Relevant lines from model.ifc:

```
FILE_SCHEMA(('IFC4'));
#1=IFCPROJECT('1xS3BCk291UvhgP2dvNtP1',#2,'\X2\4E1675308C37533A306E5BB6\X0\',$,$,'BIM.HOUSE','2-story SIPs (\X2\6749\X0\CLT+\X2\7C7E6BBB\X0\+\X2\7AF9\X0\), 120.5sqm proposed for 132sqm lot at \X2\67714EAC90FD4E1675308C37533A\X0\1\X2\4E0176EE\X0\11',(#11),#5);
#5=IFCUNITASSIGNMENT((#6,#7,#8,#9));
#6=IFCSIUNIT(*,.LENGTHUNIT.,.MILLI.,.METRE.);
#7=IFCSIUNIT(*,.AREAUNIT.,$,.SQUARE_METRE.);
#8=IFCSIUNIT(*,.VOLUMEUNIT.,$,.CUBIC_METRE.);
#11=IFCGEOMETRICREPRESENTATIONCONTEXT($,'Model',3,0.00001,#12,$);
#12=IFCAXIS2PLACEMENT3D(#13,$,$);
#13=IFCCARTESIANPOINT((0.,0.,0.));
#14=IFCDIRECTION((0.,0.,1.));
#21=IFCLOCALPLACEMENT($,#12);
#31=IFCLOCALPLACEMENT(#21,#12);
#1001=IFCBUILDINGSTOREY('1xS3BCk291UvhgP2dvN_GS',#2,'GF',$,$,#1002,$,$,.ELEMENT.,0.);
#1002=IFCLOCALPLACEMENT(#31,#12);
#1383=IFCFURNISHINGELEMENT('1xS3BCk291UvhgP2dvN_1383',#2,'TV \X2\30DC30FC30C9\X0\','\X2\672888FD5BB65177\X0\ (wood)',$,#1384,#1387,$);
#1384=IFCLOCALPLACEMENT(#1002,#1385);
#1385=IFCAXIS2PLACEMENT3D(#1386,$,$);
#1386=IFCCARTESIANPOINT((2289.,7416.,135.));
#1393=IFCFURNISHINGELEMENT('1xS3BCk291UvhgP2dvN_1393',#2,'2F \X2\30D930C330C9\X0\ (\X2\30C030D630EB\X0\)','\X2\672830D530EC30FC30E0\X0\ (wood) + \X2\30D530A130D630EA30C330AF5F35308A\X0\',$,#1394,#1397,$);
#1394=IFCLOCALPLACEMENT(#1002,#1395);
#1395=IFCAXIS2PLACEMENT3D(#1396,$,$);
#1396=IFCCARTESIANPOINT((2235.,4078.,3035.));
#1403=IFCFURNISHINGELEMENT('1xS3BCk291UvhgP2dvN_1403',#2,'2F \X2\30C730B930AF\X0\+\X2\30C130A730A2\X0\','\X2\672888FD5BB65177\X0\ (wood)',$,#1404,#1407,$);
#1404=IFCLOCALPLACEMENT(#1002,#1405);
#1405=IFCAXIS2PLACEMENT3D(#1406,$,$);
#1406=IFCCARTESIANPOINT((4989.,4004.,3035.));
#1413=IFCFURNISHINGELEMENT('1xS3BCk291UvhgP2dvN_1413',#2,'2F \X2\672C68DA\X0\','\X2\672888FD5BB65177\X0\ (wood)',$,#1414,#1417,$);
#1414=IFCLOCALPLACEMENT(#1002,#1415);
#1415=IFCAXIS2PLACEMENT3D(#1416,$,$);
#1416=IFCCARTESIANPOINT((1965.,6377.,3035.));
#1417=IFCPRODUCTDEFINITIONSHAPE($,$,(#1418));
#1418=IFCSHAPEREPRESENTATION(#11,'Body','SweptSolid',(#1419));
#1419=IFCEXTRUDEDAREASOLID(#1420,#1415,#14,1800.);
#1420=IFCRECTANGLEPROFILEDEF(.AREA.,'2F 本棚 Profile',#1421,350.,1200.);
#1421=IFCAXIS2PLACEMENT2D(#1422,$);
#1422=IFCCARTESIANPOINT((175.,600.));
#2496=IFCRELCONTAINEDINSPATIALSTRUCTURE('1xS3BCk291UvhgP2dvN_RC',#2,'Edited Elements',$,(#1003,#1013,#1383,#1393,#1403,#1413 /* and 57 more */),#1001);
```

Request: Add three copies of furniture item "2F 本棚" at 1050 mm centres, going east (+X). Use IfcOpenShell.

```python
import numpy as np
import ifcopenshell
import ifcopenshell.api.geometry
import ifcopenshell.api.root
import ifcopenshell.util.element
import ifcopenshell.util.placement
import ifcopenshell.util.unit

model = ifcopenshell.open("model.ifc")
unit_scale = ifcopenshell.util.unit.calculate_unit_scale(model)


def reuse_history(source, copy):
    """copy_class also copies each property set's owner history, people and application; keep the originals."""
    for rel in copy.IsDefinedBy:
        if rel.is_a("IfcRelDefinesByProperties") and (history := rel.RelatingPropertyDefinition.OwnerHistory):
            rel.RelatingPropertyDefinition.OwnerHistory = source.OwnerHistory
            ifcopenshell.util.element.remove_deep2(model, history)


source = model.by_id(1413)
base = ifcopenshell.util.placement.get_local_placement(source.ObjectPlacement)
step = np.array([1.0, 0.0, 0.0]) * 1.05 / unit_scale

for i in range(1, 4):
    copy = ifcopenshell.api.root.copy_class(model, product=source)
    copy.Representation = ifcopenshell.util.element.copy_deep(
        model, source.Representation, exclude=["IfcGeometricRepresentationContext", "IfcRepresentationMap"]
    )
    reuse_history(source, copy)
    matrix = base.copy()
    matrix[:3, 3] += i * step
    print("added at", matrix[:3, 3].round(3) + 0.0)
    ifcopenshell.api.geometry.edit_object_placement(model, product=copy, matrix=matrix, is_si=False)

model.write("model_updated.ifc")
```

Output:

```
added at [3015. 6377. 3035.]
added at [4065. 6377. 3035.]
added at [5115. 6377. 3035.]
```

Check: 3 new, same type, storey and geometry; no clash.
